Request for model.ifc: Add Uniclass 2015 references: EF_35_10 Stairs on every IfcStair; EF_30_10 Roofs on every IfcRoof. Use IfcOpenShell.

First a look at what the model holds.

```python
import ifcopenshell

model = ifcopenshell.open("model.ifc")
print(model.schema)
print("classifications:", [c.Name for c in model.by_type("IfcClassification")])
for ifc_class in ("IfcDoor", "IfcRoof", "IfcStair", "IfcWall", "IfcWindow"):
    print(ifc_class, len(model.by_type(ifc_class)))
```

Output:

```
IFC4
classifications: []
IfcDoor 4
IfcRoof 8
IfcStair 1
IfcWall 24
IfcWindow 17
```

```python
import ifcopenshell
import ifcopenshell.api.classification

model = ifcopenshell.open("model.ifc")

system = ifcopenshell.api.classification.add_classification(model, classification="Uniclass 2015")

codes = {
    "IfcStair": ("EF_35_10", "Stairs"),
    "IfcRoof": ("EF_30_10", "Roofs"),
}
for ifc_class, (code, name) in codes.items():
    products = model.by_type(ifc_class)
    ifcopenshell.api.classification.add_reference(
        model, products=products, classification=system, identification=code, name=name
    )
    print(code, len(products))

model.write("model_updated.ifc")
```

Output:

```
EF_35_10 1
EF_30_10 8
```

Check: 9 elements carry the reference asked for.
